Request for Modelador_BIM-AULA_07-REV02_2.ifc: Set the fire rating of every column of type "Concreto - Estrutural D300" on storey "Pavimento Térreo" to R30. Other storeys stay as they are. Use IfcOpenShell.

First a look at what the model holds.

```python
import ifcopenshell
import ifcopenshell.util.element

model = ifcopenshell.open("Modelador_BIM-AULA_07-REV02_2.ifc")
print(model.schema)
storey = next(s for s in model.by_type("IfcBuildingStorey") if s.Name == "Pavimento Térreo")
columns = [e for e in ifcopenshell.util.element.get_decomposition(storey) if e.is_a("IfcColumn")]
seen = {}
for e in columns:
    element_type = ifcopenshell.util.element.get_type(e)
    key = (element_type.Name if element_type != e and element_type else None, ifcopenshell.util.element.get_pset(e, "Pset_ColumnCommon", "FireRating"))
    seen[key] = seen.get(key, 0) + 1
for (name, value), count in sorted(seen.items(), key=str):
    print(count, "x", name, "|", value)
```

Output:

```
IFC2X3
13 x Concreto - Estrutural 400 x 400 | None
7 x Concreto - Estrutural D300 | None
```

```python
import ifcopenshell
import ifcopenshell.api.pset
import ifcopenshell.util.element

model = ifcopenshell.open("Modelador_BIM-AULA_07-REV02_2.ifc")

storey = next(s for s in model.by_type("IfcBuildingStorey") if s.Name == "Pavimento Térreo")
columns = [e for e in ifcopenshell.util.element.get_decomposition(storey) if e.is_a("IfcColumn")]

count = 0
for e in columns:
    element_type = ifcopenshell.util.element.get_type(e)
    if element_type in (None, e) or element_type.Name != "Concreto - Estrutural D300":
        continue
    # add_pset returns the element's existing set when there is one.
    pset = ifcopenshell.api.pset.add_pset(model, product=e, name="Pset_ColumnCommon")
    ifcopenshell.api.pset.edit_pset(model, pset=pset, properties={"FireRating": "R30"})
    count += 1

print(count, "columns updated")

model.write("Modelador_BIM-AULA_07-REV02_2_rev.ifc")
```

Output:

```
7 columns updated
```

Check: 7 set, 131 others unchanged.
